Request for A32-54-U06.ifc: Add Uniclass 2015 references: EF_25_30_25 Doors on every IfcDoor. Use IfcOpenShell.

First a look at what the model holds.

```python
import ifcopenshell

model = ifcopenshell.open("A32-54-U06.ifc")
print(model.schema)
print("classifications:", [c.Name for c in model.by_type("IfcClassification")])
for ifc_class in ("IfcDoor", "IfcRoof", "IfcStair", "IfcWall", "IfcWindow"):
    print(ifc_class, len(model.by_type(ifc_class)))
```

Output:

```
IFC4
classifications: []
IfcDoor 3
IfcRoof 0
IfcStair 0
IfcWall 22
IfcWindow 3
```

```python
import ifcopenshell
import ifcopenshell.api.classification

model = ifcopenshell.open("A32-54-U06.ifc")

system = ifcopenshell.api.classification.add_classification(model, classification="Uniclass 2015")

codes = {
    "IfcDoor": ("EF_25_30_25", "Doors"),
}
for ifc_class, (code, name) in codes.items():
    products = model.by_type(ifc_class)
    ifcopenshell.api.classification.add_reference(
        model, products=products, classification=system, identification=code, name=name
    )
    print(code, len(products))

model.write("A32-54-U06_updated.ifc")
```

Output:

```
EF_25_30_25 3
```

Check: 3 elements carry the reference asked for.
